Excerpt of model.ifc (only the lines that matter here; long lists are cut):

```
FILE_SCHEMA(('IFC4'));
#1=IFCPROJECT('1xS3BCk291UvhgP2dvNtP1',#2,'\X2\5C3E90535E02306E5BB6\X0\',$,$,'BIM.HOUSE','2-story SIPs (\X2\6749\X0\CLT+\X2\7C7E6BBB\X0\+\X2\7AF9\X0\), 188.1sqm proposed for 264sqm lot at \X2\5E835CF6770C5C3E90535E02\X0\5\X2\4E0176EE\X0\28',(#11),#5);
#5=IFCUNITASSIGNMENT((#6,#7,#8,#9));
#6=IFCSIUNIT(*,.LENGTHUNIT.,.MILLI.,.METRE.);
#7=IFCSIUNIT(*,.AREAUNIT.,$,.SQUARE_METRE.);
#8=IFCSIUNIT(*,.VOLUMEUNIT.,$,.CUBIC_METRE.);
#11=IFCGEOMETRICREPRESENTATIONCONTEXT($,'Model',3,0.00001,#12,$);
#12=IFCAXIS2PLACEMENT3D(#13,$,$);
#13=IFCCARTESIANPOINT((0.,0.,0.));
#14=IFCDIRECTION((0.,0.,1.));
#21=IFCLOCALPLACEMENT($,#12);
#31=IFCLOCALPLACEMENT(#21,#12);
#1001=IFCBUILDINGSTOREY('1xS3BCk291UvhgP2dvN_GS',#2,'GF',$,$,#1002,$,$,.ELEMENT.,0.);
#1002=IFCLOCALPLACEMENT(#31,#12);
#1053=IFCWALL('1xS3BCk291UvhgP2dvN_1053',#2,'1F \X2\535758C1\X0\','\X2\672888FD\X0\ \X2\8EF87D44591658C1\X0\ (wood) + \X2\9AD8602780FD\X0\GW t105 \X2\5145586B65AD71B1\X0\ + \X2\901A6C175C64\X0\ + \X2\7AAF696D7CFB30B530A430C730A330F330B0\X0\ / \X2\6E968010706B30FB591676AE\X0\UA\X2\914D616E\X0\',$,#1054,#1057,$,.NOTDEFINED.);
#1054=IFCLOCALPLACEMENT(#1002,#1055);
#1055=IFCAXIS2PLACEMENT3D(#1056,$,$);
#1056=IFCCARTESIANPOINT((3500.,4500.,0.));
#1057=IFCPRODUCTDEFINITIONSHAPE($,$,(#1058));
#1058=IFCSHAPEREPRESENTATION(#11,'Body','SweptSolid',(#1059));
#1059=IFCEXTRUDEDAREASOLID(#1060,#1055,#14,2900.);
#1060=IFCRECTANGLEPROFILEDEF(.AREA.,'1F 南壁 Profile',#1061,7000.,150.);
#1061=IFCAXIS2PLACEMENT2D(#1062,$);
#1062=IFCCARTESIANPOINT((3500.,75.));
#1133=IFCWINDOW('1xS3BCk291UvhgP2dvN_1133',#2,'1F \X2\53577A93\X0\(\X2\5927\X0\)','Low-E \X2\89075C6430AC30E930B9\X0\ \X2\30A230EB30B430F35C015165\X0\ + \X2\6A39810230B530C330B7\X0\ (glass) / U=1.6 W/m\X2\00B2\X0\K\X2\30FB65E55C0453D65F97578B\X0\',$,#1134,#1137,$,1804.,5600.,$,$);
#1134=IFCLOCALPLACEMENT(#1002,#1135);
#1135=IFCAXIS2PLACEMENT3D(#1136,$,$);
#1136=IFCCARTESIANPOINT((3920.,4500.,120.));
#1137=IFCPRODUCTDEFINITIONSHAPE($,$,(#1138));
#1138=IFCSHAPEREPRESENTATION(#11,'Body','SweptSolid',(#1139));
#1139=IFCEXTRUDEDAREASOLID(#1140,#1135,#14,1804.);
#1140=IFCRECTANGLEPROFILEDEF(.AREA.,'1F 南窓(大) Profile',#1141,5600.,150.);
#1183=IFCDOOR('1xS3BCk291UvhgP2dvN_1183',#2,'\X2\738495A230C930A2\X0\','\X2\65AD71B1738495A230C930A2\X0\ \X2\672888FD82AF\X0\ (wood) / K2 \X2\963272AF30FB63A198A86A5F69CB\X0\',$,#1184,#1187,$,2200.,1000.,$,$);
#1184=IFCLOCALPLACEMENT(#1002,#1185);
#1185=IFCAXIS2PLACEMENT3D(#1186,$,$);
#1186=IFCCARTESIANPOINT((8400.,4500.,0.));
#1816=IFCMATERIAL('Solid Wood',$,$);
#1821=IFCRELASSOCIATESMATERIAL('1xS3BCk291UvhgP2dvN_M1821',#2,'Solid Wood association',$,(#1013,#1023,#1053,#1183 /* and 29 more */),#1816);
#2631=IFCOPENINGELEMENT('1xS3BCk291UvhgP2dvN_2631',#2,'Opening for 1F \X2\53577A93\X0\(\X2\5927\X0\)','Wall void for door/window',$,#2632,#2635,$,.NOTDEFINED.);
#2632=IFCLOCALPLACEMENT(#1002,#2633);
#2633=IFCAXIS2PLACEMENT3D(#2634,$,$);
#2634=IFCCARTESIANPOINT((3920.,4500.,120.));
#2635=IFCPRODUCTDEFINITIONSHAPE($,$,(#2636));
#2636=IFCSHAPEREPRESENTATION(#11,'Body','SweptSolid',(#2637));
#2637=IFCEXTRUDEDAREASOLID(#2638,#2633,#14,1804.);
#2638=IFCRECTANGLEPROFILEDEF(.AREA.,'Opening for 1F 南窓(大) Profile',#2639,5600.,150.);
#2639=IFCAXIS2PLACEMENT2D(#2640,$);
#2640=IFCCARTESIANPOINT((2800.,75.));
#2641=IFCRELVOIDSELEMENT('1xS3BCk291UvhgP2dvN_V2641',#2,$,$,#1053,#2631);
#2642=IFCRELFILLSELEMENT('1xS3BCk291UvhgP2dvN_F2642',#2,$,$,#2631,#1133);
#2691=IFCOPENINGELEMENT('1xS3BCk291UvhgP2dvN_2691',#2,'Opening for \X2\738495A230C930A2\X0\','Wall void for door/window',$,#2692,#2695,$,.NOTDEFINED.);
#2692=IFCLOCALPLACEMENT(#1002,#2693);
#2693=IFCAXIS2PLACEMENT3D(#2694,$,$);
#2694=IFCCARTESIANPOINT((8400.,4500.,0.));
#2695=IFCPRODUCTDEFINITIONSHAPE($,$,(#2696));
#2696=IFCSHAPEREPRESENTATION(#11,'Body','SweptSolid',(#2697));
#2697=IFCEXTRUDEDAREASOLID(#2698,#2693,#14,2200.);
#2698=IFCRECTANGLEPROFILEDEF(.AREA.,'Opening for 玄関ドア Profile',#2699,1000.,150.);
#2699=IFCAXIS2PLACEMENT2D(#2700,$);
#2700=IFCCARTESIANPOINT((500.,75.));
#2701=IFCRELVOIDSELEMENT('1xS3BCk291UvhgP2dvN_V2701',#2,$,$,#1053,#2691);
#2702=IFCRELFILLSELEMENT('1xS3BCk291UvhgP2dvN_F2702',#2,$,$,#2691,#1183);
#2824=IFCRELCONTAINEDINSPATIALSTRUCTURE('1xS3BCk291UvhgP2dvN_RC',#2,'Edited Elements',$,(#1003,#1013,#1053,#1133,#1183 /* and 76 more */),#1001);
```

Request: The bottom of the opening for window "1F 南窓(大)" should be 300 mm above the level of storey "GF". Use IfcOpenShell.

```python
import numpy as np
import ifcopenshell
import ifcopenshell.api.geometry
import ifcopenshell.geom
import ifcopenshell.util.element
import ifcopenshell.util.placement
import ifcopenshell.util.shape
import ifcopenshell.util.unit

model = ifcopenshell.open("model.ifc")
unit_scale = ifcopenshell.util.unit.calculate_unit_scale(model)

window = model.by_id(1133)
opening = window.FillsVoids[0].RelatingOpeningElement
storey = ifcopenshell.util.element.get_container(window, ifc_class="IfcBuildingStorey")
level = ifcopenshell.util.placement.get_local_placement(storey.ObjectPlacement)[2, 3]

# The opening's origin need not be at the sill, so measure its lowest point.
shape = ifcopenshell.geom.create_shape(ifcopenshell.geom.settings(), opening)
bottom = ifcopenshell.util.shape.get_shape_bottom_elevation(shape, shape.geometry) / unit_scale
dz = level + 0.3 / unit_scale - bottom

shift = np.array([0.0, 0.0, dz])
# The window is not placed relative to its opening, so move both.
for product in (opening, window):
    matrix = ifcopenshell.util.placement.get_local_placement(product.ObjectPlacement)
    matrix[:3, 3] += shift
    ifcopenshell.api.geometry.edit_object_placement(model, product=product, matrix=matrix, is_si=False)

print(f"moved by {dz * unit_scale:+.3f} m")

model.write("model_rev.ifc")
```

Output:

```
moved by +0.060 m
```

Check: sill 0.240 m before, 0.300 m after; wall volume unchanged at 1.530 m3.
